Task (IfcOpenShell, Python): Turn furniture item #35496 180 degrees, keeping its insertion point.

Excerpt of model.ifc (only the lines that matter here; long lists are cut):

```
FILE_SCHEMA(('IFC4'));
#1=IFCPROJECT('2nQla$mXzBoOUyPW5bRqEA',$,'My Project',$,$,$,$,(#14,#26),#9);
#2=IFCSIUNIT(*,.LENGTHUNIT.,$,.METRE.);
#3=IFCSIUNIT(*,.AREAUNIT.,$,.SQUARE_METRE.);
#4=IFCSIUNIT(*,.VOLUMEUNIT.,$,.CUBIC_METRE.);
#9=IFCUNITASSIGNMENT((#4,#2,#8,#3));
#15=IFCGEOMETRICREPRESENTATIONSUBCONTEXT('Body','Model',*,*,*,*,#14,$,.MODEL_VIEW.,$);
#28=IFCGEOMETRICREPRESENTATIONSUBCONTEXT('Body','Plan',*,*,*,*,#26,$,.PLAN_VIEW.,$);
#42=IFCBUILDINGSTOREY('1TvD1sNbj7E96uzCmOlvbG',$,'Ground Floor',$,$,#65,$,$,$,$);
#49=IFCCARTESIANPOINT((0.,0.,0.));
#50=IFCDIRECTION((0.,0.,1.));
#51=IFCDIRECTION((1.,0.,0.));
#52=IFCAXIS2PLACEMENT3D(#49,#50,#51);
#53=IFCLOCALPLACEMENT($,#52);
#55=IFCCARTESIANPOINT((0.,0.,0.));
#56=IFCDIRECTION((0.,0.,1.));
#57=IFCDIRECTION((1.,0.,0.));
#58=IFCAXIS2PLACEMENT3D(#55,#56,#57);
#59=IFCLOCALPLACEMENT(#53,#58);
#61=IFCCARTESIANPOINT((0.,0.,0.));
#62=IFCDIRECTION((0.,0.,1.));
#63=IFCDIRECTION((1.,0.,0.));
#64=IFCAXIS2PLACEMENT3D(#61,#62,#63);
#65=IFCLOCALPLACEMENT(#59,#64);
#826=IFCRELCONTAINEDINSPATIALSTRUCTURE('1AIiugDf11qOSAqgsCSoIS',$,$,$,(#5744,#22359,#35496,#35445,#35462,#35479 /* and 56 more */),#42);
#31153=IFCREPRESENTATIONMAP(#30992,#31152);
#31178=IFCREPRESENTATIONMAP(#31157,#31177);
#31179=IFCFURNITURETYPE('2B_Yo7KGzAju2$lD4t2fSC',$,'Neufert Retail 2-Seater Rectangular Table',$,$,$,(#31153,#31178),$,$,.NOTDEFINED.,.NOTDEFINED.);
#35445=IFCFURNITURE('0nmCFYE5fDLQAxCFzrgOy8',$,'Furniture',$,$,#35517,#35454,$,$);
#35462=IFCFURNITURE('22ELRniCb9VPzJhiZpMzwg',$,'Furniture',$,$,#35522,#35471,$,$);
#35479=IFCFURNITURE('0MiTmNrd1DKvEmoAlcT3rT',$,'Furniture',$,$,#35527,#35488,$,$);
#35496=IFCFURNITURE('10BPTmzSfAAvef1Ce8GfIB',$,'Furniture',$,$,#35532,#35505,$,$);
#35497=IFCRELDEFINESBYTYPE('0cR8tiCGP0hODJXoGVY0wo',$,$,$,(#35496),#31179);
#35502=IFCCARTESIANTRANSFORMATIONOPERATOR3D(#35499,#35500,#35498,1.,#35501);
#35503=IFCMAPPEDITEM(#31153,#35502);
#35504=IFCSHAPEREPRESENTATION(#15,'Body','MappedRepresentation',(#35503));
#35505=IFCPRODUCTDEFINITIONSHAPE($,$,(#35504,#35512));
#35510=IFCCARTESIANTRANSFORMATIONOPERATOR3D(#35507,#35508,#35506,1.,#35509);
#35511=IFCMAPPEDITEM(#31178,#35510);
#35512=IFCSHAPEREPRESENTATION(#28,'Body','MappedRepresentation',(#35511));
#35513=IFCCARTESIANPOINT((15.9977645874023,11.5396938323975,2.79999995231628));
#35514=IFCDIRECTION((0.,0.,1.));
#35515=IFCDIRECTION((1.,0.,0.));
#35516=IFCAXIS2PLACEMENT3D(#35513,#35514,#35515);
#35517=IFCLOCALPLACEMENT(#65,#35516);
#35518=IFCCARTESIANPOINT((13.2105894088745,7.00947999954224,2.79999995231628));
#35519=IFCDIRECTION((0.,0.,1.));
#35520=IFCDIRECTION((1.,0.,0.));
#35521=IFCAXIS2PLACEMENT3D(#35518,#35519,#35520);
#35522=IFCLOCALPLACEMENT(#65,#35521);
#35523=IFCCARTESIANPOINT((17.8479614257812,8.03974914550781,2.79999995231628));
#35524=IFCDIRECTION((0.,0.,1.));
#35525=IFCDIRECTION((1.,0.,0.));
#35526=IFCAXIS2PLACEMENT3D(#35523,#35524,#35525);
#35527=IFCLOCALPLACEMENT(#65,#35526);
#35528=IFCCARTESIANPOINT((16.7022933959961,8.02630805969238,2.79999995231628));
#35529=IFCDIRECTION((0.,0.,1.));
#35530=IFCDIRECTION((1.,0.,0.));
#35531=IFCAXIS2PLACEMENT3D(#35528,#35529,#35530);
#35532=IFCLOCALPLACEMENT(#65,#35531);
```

```python
import ifcopenshell
import ifcopenshell.api.geometry
import ifcopenshell.util.placement

model = ifcopenshell.open("model.ifc")

item = model.by_guid("10BPTmzSfAAvef1Ce8GfIB")
matrix = ifcopenshell.util.placement.get_local_placement(item.ObjectPlacement)
matrix = matrix @ ifcopenshell.util.placement.rotation(180, "Z")
ifcopenshell.api.geometry.edit_object_placement(model, product=item, matrix=matrix, is_si=False)

print(ifcopenshell.util.placement.get_local_placement(item.ObjectPlacement).round(3) + 0.0)

model.write("model_updated.ifc")
```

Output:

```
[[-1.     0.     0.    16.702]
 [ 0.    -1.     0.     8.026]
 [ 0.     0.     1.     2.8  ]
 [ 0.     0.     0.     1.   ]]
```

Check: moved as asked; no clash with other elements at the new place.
